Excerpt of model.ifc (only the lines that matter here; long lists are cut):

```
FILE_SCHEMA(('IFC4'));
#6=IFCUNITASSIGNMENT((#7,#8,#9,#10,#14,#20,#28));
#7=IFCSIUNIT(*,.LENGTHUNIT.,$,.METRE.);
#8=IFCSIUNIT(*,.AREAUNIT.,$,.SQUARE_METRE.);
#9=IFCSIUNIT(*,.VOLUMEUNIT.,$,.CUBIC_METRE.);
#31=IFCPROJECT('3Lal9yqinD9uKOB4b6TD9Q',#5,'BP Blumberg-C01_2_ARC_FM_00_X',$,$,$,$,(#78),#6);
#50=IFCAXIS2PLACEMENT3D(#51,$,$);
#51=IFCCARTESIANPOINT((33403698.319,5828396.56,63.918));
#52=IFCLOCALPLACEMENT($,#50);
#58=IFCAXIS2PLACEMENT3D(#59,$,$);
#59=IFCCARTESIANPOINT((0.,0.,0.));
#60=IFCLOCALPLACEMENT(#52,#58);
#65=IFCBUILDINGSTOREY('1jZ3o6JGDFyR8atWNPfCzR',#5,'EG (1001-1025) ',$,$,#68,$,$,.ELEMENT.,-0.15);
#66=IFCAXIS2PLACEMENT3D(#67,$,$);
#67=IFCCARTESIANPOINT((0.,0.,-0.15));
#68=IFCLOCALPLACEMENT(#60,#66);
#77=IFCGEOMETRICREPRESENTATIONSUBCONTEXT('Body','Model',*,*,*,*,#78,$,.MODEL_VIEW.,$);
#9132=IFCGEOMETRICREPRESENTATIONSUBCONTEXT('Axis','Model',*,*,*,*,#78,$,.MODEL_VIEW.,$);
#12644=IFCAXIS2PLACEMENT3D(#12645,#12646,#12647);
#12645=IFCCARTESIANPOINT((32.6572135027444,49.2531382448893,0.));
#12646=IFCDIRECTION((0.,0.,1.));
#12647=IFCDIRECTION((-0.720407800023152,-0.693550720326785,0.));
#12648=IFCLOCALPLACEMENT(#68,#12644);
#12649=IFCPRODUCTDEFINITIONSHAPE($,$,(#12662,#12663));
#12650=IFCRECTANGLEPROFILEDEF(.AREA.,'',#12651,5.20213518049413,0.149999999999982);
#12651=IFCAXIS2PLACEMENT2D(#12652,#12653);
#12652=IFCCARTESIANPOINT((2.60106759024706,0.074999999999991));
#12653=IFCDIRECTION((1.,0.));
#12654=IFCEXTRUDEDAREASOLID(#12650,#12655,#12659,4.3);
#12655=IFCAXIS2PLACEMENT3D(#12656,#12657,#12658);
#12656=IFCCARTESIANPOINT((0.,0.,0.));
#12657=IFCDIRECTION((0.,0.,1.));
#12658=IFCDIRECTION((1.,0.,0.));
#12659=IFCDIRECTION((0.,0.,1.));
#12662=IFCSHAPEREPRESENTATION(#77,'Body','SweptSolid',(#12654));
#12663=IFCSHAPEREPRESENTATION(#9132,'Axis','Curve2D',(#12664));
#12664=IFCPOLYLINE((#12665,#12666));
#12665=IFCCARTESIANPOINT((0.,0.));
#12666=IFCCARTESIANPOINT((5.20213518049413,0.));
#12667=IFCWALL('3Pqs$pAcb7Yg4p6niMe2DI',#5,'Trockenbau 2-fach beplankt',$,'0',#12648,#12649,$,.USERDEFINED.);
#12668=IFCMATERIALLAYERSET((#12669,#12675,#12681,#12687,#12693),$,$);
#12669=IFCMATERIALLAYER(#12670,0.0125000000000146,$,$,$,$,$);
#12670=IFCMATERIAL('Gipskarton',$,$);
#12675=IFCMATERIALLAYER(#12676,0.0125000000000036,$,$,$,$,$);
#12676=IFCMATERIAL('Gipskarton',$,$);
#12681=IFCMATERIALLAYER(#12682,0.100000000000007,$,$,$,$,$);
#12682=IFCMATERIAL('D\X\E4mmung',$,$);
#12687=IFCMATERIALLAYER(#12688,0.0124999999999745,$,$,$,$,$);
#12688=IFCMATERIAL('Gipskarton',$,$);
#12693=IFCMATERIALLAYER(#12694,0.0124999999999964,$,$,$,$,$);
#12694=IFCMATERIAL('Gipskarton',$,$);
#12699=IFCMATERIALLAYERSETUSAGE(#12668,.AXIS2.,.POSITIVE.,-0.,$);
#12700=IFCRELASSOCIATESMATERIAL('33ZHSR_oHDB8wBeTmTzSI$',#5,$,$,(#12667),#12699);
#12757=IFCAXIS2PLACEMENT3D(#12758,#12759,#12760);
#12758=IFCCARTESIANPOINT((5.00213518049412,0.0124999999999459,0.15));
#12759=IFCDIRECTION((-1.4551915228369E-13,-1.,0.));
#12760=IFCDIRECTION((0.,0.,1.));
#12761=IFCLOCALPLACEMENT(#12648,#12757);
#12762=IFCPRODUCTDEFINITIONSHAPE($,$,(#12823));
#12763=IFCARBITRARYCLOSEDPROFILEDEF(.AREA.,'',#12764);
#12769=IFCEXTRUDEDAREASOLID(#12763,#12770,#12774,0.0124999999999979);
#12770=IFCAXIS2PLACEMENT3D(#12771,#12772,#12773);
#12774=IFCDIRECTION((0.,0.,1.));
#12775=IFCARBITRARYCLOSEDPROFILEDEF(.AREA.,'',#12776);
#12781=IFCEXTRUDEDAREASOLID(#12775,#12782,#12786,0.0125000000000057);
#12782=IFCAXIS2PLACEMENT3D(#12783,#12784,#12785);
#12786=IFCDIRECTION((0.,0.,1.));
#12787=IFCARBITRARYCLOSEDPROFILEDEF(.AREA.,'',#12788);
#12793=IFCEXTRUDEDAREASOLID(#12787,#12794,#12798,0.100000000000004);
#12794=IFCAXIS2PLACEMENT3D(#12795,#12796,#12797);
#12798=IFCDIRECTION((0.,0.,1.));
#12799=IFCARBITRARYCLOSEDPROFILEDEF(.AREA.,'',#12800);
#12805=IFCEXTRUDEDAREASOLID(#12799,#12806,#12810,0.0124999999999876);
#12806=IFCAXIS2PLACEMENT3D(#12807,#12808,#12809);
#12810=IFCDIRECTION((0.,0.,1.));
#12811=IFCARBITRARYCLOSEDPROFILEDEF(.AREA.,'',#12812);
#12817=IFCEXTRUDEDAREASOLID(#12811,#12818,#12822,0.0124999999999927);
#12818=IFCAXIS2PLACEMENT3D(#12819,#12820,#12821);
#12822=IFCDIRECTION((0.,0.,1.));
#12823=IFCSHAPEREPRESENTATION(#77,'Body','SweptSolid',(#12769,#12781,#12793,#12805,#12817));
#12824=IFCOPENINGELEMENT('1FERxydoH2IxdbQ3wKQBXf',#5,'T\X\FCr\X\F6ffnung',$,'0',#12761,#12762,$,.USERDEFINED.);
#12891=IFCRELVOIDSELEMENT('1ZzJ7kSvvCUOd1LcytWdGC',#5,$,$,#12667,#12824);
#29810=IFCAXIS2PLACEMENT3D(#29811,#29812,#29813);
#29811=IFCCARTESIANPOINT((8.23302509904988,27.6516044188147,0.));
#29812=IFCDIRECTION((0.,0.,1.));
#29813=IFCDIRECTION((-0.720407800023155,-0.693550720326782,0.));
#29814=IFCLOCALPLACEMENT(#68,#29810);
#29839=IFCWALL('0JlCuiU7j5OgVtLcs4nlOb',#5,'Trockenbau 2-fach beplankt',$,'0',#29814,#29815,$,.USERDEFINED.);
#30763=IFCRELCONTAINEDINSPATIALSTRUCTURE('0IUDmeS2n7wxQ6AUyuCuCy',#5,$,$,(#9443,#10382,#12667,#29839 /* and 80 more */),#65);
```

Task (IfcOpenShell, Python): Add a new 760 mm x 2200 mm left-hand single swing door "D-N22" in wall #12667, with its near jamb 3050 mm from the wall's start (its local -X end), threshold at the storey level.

```python
import numpy as np
import ifcopenshell
import ifcopenshell.api.feature
import ifcopenshell.api.geometry
import ifcopenshell.api.root
import ifcopenshell.api.spatial
import ifcopenshell.geom
import ifcopenshell.util.element
import ifcopenshell.util.placement
import ifcopenshell.util.representation
import ifcopenshell.util.shape
import ifcopenshell.util.unit

model = ifcopenshell.open("model.ifc")
unit_scale = ifcopenshell.util.unit.calculate_unit_scale(model)
settings = ifcopenshell.geom.settings()


def volume(element):
    """Net volume in cubic metres, openings subtracted."""
    shape = ifcopenshell.geom.create_shape(settings, element)
    return ifcopenshell.util.shape.get_volume(shape.geometry)


wall = model.by_guid("3Pqs$pAcb7Yg4p6niMe2DI")
storey = ifcopenshell.util.element.get_container(wall, ifc_class="IfcBuildingStorey")
context = ifcopenshell.util.representation.get_context(model, "Model", "Body", "MODEL_VIEW")
before = volume(wall)

width, height, from_end, sill = 0.76, 2.2, 3.05, 0.0  # metres

# The wall runs along its own X axis, and the end named is its -X end.
wall_shape = ifcopenshell.geom.create_shape(settings, wall)
x, y, z = ifcopenshell.util.shape.get_vertices(wall_shape.geometry).T
start = x.min() + from_end
face, thickness = float(y.min()), float(y.max() - y.min())
wall_matrix = ifcopenshell.util.placement.get_local_placement(wall.ObjectPlacement)
level = ifcopenshell.util.placement.get_local_placement(storey.ObjectPlacement)[2, 3]


def in_wall(x, y):
    """Placement at x, y metres in the wall's axes, at sill height."""
    matrix = wall_matrix.copy()
    matrix[:, 3] = wall_matrix @ np.array([x / unit_scale, y / unit_scale, 0.0, 1.0])
    matrix[2, 3] = level + sill / unit_scale
    return matrix


# Opening: a box that overshoots both wall faces by 50 mm.
opening = ifcopenshell.api.root.create_entity(model, ifc_class="IfcOpeningElement", predefined_type="OPENING")
box = ifcopenshell.api.geometry.add_wall_representation(
    model, context=context, length=width, height=height, thickness=thickness + 0.1
)
ifcopenshell.api.geometry.assign_representation(model, product=opening, representation=box)
ifcopenshell.api.geometry.edit_object_placement(model, product=opening, matrix=in_wall(start, face - 0.05), is_si=False)
ifcopenshell.api.feature.add_feature(model, feature=opening, element=wall)

door = ifcopenshell.api.root.create_entity(model, ifc_class="IfcDoor", name="D-N22", predefined_type="DOOR")
door.OverallWidth, door.OverallHeight = width / unit_scale, height / unit_scale
door.OperationType = "SINGLE_SWING_LEFT"
body = ifcopenshell.api.geometry.add_door_representation(
    model,
    context=context,
    overall_width=door.OverallWidth,
    overall_height=door.OverallHeight,
    operation_type="SINGLE_SWING_LEFT",
    lining_properties={"LiningDepth": thickness / unit_scale, "ThresholdDepth": thickness / unit_scale},
)
ifcopenshell.api.geometry.assign_representation(model, product=door, representation=body)
ifcopenshell.api.spatial.assign_container(model, products=[door], relating_structure=storey)
ifcopenshell.api.feature.add_filling(model, opening=opening, element=door)

# The lining spans the wall, so the door starts at the wall face.
ifcopenshell.api.geometry.edit_object_placement(model, product=door, matrix=in_wall(start, face), is_si=False)

after = volume(wall)

print(f"wall volume {before:.3f} -> {after:.3f} m3")

model.write("model_rev.ifc")
```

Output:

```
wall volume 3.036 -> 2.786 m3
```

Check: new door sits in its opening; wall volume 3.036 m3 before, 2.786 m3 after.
